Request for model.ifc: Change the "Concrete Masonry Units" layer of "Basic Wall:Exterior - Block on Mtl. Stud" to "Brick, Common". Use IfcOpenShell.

First a look at what the model holds.

```python
import ifcopenshell
import ifcopenshell.util.element

model = ifcopenshell.open("model.ifc")
print(model.schema)
for layer_set in model.by_type("IfcMaterialLayerSet"):
    if layer_set.LayerSetName == "Basic Wall:Exterior - Block on Mtl. Stud":
        for layer in layer_set.MaterialLayers:
            print(layer.id(), layer.Material and layer.Material.Name, layer.LayerThickness, sep=" | ")
        print(len(ifcopenshell.util.element.get_elements_by_material(model, layer_set)), "elements and types use it")
print(sorted(m.Name for m in model.by_type("IfcMaterial") if m.Name)[:60])
```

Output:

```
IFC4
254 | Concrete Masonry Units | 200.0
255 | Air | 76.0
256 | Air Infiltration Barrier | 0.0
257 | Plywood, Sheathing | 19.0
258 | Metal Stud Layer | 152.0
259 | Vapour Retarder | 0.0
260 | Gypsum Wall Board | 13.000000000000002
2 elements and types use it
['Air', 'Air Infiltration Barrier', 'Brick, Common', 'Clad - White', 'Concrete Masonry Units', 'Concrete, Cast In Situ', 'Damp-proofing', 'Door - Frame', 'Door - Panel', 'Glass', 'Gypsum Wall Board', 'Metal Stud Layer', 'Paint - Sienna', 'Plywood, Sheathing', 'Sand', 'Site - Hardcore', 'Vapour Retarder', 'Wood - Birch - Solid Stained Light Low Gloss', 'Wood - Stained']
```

```python
import ifcopenshell
import ifcopenshell.api.material

model = ifcopenshell.open("model.ifc")

layer_set = next(s for s in model.by_type("IfcMaterialLayerSet") if s.LayerSetName == "Basic Wall:Exterior - Block on Mtl. Stud")
layer = next(l for l in layer_set.MaterialLayers if l.Material and l.Material.Name == "Concrete Masonry Units")
material = next(m for m in model.by_type("IfcMaterial") if m.Name == "Brick, Common")

# Point this one layer at the other material; renaming the old one would change it everywhere.
ifcopenshell.api.material.edit_layer(model, layer=layer, attributes={"Name": material.Name}, material=material)

print([l.Material.Name if l.Material else None for l in layer_set.MaterialLayers])

model.write("model_rev.ifc")
```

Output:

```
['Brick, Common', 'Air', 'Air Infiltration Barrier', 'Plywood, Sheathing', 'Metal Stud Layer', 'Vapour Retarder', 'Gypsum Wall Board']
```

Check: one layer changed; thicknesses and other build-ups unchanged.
